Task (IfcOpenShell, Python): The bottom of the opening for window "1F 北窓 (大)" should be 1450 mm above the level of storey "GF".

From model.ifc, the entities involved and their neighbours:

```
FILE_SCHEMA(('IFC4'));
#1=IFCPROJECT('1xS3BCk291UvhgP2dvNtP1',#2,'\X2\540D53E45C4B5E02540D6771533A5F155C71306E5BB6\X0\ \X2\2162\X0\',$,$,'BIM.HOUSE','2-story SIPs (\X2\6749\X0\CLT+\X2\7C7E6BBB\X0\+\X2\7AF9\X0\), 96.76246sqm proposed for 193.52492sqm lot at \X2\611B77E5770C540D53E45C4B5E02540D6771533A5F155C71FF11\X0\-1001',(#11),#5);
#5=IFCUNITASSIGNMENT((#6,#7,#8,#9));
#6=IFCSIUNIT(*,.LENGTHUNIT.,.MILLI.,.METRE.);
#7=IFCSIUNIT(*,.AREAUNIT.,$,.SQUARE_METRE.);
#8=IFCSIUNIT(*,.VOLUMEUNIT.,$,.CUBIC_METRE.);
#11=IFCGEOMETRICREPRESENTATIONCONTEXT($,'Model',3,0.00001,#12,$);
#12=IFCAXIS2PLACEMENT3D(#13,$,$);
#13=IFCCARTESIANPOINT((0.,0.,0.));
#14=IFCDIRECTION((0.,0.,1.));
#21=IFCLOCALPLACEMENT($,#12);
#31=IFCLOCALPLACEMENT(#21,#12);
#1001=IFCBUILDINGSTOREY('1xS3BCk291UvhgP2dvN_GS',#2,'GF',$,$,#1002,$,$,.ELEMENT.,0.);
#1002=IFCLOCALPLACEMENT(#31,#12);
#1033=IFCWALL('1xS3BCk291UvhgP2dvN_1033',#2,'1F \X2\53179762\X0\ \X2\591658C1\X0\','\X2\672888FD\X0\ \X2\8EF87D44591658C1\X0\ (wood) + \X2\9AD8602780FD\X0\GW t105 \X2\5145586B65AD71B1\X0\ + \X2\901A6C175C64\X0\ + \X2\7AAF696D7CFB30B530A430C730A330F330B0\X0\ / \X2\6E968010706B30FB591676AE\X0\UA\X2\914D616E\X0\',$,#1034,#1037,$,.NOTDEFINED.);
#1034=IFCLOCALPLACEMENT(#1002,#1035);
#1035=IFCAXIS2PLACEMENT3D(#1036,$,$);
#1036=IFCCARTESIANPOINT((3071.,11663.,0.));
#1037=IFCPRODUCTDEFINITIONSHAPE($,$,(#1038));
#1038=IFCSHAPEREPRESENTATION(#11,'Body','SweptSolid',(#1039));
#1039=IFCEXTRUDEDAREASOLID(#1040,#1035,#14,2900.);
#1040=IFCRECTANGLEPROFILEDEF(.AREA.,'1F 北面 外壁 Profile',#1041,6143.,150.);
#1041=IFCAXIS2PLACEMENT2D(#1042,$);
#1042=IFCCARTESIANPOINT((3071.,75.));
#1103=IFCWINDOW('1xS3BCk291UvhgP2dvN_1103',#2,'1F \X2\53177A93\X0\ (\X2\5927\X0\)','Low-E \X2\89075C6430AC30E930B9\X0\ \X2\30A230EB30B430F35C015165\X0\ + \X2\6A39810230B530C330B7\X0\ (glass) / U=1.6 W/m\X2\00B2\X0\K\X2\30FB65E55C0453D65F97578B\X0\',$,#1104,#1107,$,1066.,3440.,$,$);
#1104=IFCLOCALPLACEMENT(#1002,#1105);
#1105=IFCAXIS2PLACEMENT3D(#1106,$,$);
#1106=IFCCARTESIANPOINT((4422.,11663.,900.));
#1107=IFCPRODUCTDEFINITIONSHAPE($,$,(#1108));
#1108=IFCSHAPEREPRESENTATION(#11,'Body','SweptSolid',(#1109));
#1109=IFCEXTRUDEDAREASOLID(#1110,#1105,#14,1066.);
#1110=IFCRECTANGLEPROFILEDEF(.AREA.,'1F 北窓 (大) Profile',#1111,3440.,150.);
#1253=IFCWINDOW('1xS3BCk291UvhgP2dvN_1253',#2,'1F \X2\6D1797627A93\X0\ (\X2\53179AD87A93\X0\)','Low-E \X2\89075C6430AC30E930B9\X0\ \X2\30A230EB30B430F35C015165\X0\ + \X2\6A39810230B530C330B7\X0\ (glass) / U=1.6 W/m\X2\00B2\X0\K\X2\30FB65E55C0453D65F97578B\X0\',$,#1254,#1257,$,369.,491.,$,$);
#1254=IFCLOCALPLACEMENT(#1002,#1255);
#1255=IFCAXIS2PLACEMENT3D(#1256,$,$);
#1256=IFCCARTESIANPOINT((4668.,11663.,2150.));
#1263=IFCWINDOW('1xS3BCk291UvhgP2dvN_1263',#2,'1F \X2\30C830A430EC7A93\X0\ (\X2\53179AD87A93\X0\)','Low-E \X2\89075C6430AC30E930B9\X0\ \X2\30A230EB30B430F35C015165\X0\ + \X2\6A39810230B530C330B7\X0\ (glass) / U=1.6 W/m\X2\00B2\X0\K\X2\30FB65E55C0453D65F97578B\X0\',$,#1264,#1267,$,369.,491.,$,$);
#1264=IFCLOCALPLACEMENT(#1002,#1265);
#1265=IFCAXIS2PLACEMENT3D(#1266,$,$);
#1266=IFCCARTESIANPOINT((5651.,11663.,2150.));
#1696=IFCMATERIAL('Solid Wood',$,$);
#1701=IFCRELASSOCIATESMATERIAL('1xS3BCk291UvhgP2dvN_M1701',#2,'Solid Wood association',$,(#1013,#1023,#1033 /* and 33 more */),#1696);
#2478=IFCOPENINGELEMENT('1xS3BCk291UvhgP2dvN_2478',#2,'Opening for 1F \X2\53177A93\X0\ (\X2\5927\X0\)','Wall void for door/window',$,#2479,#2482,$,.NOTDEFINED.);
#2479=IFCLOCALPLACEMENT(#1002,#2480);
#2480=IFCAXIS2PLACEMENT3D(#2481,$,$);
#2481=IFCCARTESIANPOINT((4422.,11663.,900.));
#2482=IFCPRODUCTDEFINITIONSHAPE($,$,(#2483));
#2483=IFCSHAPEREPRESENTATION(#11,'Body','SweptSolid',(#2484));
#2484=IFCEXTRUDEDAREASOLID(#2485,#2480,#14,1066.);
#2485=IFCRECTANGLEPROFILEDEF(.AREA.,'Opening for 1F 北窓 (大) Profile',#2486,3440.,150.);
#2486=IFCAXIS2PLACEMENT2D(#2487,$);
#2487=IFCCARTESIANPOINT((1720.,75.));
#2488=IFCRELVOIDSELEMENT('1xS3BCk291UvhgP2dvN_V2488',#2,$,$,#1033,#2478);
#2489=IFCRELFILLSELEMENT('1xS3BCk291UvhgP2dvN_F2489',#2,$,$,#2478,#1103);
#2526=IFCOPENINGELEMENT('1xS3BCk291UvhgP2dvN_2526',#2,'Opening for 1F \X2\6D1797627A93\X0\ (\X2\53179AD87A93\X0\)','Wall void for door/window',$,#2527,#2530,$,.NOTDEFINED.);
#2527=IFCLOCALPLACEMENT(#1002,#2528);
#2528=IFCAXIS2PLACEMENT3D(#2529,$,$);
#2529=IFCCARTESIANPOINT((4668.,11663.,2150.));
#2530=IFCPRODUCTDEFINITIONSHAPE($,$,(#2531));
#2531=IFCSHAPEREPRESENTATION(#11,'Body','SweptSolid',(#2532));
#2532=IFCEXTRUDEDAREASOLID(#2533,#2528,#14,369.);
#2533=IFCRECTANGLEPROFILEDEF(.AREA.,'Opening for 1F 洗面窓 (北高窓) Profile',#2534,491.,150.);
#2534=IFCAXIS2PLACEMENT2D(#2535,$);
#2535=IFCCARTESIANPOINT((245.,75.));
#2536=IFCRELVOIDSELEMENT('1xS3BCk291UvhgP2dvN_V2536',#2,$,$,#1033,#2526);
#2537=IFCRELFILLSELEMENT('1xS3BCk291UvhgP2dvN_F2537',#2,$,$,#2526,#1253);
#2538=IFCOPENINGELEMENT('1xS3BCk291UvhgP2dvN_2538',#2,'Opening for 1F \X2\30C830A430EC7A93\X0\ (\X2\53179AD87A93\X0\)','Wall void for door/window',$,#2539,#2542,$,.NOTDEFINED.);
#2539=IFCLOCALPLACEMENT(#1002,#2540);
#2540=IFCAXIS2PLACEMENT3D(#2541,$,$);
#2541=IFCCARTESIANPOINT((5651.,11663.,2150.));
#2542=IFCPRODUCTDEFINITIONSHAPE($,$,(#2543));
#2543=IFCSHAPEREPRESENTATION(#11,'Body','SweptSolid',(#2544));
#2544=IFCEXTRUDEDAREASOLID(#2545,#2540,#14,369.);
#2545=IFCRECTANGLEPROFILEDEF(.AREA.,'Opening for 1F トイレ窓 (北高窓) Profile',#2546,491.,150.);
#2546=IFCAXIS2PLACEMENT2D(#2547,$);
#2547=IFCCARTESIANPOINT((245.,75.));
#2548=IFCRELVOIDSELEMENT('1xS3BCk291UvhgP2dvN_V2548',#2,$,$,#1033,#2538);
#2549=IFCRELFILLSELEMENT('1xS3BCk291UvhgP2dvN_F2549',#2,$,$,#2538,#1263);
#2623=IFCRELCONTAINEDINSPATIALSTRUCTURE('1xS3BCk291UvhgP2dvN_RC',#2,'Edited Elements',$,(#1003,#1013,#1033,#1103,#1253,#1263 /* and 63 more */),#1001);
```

```python
import numpy as np
import ifcopenshell
import ifcopenshell.api.geometry
import ifcopenshell.geom
import ifcopenshell.util.element
import ifcopenshell.util.placement
import ifcopenshell.util.shape
import ifcopenshell.util.unit

model = ifcopenshell.open("model.ifc")
unit_scale = ifcopenshell.util.unit.calculate_unit_scale(model)

window = model.by_guid("1xS3BCk291UvhgP2dvN_1103")
opening = window.FillsVoids[0].RelatingOpeningElement
storey = ifcopenshell.util.element.get_container(window, ifc_class="IfcBuildingStorey")
level = ifcopenshell.util.placement.get_local_placement(storey.ObjectPlacement)[2, 3]

# The opening's origin need not be at the sill, so measure its lowest point.
shape = ifcopenshell.geom.create_shape(ifcopenshell.geom.settings(), opening)
bottom = ifcopenshell.util.shape.get_shape_bottom_elevation(shape, shape.geometry) / unit_scale
dz = level + 1.45 / unit_scale - bottom

shift = np.array([0.0, 0.0, dz])
# The window is not placed relative to its opening, so move both.
for product in (opening, window):
    matrix = ifcopenshell.util.placement.get_local_placement(product.ObjectPlacement)
    matrix[:3, 3] += shift
    ifcopenshell.api.geometry.edit_object_placement(model, product=product, matrix=matrix, is_si=False)

print(f"moved by {dz * unit_scale:+.3f} m")

model.write("model_updated.ifc")
```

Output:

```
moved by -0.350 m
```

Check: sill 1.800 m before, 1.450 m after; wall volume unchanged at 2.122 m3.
